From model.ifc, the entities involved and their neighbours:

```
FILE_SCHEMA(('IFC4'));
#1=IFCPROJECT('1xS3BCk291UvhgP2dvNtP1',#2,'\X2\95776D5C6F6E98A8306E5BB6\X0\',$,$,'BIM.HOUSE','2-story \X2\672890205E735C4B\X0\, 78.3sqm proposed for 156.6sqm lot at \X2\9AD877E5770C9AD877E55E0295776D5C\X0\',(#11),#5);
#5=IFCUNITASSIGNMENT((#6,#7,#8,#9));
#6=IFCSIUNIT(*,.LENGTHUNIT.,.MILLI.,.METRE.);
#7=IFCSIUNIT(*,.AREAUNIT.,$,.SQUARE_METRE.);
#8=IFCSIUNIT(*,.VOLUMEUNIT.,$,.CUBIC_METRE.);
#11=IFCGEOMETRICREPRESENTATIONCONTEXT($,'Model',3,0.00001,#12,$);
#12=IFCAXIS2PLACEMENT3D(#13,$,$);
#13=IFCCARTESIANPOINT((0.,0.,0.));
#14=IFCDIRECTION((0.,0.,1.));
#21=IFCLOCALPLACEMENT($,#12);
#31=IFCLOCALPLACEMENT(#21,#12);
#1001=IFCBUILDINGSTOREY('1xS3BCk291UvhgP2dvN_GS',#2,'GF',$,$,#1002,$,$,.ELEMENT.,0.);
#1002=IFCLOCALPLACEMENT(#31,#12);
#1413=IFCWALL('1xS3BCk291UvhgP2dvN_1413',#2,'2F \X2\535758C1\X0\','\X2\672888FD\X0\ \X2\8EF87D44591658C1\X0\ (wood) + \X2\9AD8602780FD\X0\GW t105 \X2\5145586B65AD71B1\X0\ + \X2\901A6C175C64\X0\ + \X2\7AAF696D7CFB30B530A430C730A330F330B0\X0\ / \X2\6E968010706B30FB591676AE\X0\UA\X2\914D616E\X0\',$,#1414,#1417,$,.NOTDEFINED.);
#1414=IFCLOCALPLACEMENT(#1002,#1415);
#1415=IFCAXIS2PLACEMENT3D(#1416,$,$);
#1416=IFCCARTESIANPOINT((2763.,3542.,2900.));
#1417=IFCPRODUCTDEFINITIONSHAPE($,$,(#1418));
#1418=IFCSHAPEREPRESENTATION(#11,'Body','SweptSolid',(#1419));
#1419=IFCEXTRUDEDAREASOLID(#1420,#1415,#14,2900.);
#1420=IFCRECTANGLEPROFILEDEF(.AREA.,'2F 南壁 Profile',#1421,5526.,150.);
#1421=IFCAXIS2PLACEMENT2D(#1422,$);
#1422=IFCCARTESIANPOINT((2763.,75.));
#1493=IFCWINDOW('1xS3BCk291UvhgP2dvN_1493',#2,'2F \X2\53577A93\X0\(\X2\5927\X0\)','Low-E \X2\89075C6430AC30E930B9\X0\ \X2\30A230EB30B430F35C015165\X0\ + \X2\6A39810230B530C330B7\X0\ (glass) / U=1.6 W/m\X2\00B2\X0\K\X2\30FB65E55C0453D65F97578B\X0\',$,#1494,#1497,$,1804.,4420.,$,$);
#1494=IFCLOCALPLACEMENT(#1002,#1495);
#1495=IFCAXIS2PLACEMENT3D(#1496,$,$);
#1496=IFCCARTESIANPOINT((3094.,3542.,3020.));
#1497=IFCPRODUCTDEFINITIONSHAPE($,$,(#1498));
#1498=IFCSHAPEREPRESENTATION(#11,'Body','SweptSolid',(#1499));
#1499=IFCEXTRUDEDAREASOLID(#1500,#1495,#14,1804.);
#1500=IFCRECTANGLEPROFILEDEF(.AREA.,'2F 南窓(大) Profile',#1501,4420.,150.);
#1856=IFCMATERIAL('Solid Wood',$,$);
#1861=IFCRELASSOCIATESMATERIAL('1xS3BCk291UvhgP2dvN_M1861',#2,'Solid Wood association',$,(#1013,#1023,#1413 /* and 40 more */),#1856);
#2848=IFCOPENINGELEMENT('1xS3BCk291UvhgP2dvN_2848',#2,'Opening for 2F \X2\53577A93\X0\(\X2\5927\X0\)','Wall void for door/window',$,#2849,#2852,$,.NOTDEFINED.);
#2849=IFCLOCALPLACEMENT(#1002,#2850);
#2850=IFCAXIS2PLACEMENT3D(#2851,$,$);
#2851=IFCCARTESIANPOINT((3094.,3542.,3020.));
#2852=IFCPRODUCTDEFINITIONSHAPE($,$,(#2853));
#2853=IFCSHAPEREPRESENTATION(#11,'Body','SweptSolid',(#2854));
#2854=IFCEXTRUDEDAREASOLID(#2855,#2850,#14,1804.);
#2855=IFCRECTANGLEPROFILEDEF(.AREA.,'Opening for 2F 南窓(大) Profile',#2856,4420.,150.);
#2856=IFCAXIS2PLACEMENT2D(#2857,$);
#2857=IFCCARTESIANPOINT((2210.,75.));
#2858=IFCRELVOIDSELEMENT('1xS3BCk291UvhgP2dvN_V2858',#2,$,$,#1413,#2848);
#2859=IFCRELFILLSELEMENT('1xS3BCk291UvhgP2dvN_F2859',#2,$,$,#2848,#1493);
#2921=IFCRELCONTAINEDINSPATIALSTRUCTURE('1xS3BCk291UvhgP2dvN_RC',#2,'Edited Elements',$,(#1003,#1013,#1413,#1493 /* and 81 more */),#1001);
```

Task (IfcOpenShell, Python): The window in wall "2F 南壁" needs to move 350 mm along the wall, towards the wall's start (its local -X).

```python
import ifcopenshell
import ifcopenshell.api.geometry
import ifcopenshell.util.placement
import ifcopenshell.util.unit

model = ifcopenshell.open("model.ifc")
unit_scale = ifcopenshell.util.unit.calculate_unit_scale(model)

window = model.by_guid("1xS3BCk291UvhgP2dvN_1493")
opening = window.FillsVoids[0].RelatingOpeningElement
wall = opening.VoidsElements[0].RelatingBuildingElement

wall_matrix = ifcopenshell.util.placement.get_local_placement(wall.ObjectPlacement)
shift = wall_matrix[:3, 0] * -0.35 / unit_scale
before = ifcopenshell.util.placement.get_local_placement(window.ObjectPlacement)[:3, 3].copy()

# The window is not placed relative to its opening, so move both.
for product in (opening, window):
    matrix = ifcopenshell.util.placement.get_local_placement(product.ObjectPlacement)
    matrix[:3, 3] += shift
    ifcopenshell.api.geometry.edit_object_placement(model, product=product, matrix=matrix, is_si=False)

after = ifcopenshell.util.placement.get_local_placement(window.ObjectPlacement)[:3, 3]
print("window moved by", (after - before).round(3) + 0.0)

model.write("model_updated.ifc")
```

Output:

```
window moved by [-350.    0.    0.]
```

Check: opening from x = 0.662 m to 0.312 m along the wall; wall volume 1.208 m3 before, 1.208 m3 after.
